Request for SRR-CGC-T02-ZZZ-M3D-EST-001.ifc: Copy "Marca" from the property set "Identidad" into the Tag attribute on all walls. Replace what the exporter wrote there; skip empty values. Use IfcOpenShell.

First a look at what the model holds.

```python
import ifcopenshell
import ifcopenshell.util.element

model = ifcopenshell.open("SRR-CGC-T02-ZZZ-M3D-EST-001.ifc")
print(model.schema)
walls = model.by_type("IfcWall")
print(len(walls), "walls")
for e in walls[:8]:
    source = ifcopenshell.util.element.get_pset(e, "Identidad", "Marca")
    target = e.Tag
    print(e.id(), repr(source), repr(target), sep=" | ")
```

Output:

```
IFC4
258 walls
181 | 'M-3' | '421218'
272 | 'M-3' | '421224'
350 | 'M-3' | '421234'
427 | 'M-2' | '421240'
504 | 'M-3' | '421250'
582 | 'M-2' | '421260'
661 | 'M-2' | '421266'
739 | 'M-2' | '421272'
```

```python
import ifcopenshell
import ifcopenshell.util.element

model = ifcopenshell.open("SRR-CGC-T02-ZZZ-M3D-EST-001.ifc")

count = 0
for e in model.by_type("IfcWall"):
    value = ifcopenshell.util.element.get_pset(e, "Identidad", "Marca")
    current = e.Tag
    if not value or not value.strip() or current == value:
        continue
    e.Tag = value
    count += 1

print(count, "walls updated")

model.write("SRR-CGC-T02-ZZZ-M3D-EST-001-out.ifc")
```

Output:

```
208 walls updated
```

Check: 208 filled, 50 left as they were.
